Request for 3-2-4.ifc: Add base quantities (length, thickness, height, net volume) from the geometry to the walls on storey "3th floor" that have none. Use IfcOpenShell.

First a look at what the model holds.

```python
import ifcopenshell
import ifcopenshell.util.element
import ifcopenshell.util.unit

model = ifcopenshell.open("3-2-4.ifc")
print(model.schema)
for unit_type in ("LENGTHUNIT", "AREAUNIT", "VOLUMEUNIT"):
    print(unit_type, ifcopenshell.util.unit.calculate_unit_scale(model, unit_type))
storey = next(s for s in model.by_type("IfcBuildingStorey") if s.Name == "3th floor")
walls = [e for e in ifcopenshell.util.element.get_decomposition(storey) if e.is_a("IfcWall")]
for e in sorted(walls, key=lambda e: e.id()):
    print(e.id(), e.is_a(), e.Name, list(ifcopenshell.util.element.get_psets(e, qtos_only=True)), sep=" | ")
```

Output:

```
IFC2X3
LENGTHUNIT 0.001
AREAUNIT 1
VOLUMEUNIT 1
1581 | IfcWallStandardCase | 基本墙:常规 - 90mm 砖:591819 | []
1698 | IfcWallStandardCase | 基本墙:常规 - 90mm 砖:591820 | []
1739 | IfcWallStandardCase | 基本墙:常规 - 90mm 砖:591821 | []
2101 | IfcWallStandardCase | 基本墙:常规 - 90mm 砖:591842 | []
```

```python
import ifcopenshell
import ifcopenshell.api.pset
import ifcopenshell.geom
import ifcopenshell.util.element
import ifcopenshell.util.shape
import ifcopenshell.util.unit

model = ifcopenshell.open("3-2-4.ifc")
unit_scale = ifcopenshell.util.unit.calculate_unit_scale(model)
volume_scale = ifcopenshell.util.unit.calculate_unit_scale(model, "VOLUMEUNIT")
settings = ifcopenshell.geom.settings()

storey = next(s for s in model.by_type("IfcBuildingStorey") if s.Name == "3th floor")
walls = [e for e in ifcopenshell.util.element.get_decomposition(storey) if e.is_a("IfcWall")]

for e in sorted(walls, key=lambda e: e.id()):
    if ifcopenshell.util.element.get_psets(e, qtos_only=True, should_inherit=False):
        continue
    # Geometry comes back in metres, in the element's own axes.
    shape = ifcopenshell.geom.create_shape(settings, e)
    values = {
        "Length": ifcopenshell.util.shape.get_x(shape.geometry) / unit_scale,
        "Width": ifcopenshell.util.shape.get_y(shape.geometry) / unit_scale,
        "Height": ifcopenshell.util.shape.get_z(shape.geometry) / unit_scale,
        "NetVolume": ifcopenshell.util.shape.get_volume(shape.geometry) / volume_scale,
    }
    qto = ifcopenshell.api.pset.add_qto(model, product=e, name="BaseQuantities")
    ifcopenshell.api.pset.edit_qto(model, qto=qto, properties=values)
    print(e.id(), {k: round(v, 3) for k, v in values.items()})

model.write("3-2-4_v2.ifc")
```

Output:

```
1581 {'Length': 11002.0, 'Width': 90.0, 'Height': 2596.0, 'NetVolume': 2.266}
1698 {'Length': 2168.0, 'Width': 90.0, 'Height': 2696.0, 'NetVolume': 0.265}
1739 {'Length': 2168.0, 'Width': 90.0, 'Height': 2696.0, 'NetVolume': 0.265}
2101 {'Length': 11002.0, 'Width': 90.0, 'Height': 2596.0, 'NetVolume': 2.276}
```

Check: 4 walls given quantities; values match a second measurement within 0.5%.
